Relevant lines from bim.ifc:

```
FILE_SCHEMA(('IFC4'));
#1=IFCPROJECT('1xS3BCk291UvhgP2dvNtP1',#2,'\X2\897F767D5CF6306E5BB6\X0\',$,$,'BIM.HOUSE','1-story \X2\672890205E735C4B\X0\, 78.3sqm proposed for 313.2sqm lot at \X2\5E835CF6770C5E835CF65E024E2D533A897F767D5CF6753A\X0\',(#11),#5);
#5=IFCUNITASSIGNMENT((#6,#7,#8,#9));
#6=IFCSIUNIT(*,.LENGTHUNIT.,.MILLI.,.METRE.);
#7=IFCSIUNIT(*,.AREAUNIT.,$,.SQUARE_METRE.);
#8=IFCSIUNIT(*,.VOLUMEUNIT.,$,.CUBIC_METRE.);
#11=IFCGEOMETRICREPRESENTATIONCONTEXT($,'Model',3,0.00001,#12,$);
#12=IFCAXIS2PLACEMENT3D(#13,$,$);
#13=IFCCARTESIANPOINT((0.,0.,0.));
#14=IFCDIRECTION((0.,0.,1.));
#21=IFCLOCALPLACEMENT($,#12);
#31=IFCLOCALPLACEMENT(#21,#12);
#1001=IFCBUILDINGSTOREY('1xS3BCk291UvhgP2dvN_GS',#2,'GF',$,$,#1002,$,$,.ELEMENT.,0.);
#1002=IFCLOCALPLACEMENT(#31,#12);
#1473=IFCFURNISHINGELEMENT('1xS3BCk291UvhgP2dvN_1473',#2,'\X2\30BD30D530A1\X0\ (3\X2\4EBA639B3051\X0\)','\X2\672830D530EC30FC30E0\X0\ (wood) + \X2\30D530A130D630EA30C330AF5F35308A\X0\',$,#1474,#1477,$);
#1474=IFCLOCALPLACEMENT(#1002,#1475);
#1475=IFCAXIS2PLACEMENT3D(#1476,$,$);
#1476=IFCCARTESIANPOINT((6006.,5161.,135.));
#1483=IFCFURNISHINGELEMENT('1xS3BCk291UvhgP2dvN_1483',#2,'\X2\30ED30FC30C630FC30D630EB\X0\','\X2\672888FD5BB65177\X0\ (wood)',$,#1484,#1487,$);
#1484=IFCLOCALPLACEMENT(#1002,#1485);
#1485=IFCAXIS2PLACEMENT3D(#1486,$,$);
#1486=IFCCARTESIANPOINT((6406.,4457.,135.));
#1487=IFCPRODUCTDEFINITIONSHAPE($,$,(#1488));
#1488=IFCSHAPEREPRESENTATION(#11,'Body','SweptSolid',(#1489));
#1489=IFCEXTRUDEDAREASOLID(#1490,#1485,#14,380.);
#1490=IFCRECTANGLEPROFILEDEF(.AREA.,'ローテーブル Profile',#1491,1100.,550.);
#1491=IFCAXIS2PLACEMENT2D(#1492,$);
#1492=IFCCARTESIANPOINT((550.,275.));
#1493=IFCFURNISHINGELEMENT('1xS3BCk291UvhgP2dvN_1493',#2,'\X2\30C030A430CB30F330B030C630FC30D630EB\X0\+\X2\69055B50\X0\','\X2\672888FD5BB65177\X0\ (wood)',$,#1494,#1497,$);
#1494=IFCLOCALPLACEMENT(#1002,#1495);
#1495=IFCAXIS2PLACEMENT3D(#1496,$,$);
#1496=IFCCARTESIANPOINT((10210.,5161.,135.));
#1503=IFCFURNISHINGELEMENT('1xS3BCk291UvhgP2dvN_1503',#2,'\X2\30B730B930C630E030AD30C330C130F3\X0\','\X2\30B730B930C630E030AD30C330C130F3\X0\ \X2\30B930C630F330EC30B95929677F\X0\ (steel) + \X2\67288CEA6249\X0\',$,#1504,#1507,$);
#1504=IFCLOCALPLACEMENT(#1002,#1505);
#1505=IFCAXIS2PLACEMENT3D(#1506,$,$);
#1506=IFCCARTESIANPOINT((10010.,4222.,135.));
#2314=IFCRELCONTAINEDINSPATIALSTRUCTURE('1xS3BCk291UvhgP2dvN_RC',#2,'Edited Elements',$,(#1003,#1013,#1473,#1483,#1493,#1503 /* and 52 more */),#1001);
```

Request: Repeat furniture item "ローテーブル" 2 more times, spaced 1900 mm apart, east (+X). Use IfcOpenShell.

```python
import numpy as np
import ifcopenshell
import ifcopenshell.api.geometry
import ifcopenshell.api.root
import ifcopenshell.util.element
import ifcopenshell.util.placement

model = ifcopenshell.open("bim.ifc")


def reuse_history(source, copy):
    """copy_class also copies each property set's owner history, people and application; keep the originals."""
    for rel in copy.IsDefinedBy:
        if rel.is_a("IfcRelDefinesByProperties") and (history := rel.RelatingPropertyDefinition.OwnerHistory):
            rel.RelatingPropertyDefinition.OwnerHistory = source.OwnerHistory
            ifcopenshell.util.element.remove_deep2(model, history)


source = model.by_guid("1xS3BCk291UvhgP2dvN_1483")
base = ifcopenshell.util.placement.get_local_placement(source.ObjectPlacement)
step = np.array([1.0, 0.0, 0.0]) * 1900.0

for i in range(1, 3):
    copy = ifcopenshell.api.root.copy_class(model, product=source)
    copy.Representation = ifcopenshell.util.element.copy_deep(
        model, source.Representation, exclude=["IfcGeometricRepresentationContext", "IfcRepresentationMap"]
    )
    reuse_history(source, copy)
    matrix = base.copy()
    matrix[:3, 3] += i * step
    print("added at", matrix[:3, 3].round(3) + 0.0)
    ifcopenshell.api.geometry.edit_object_placement(model, product=copy, matrix=matrix, is_si=False)

model.write("bim_v2.ifc")
```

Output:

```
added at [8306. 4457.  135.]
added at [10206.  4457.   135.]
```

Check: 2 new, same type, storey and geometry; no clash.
